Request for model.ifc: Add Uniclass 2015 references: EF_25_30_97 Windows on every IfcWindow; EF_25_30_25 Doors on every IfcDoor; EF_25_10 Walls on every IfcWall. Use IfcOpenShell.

First a look at what the model holds.

```python
import ifcopenshell

model = ifcopenshell.open("model.ifc")
print(model.schema)
print("classifications:", [c.Name for c in model.by_type("IfcClassification")])
for ifc_class in ("IfcDoor", "IfcRoof", "IfcStair", "IfcWall", "IfcWindow"):
    print(ifc_class, len(model.by_type(ifc_class)))
```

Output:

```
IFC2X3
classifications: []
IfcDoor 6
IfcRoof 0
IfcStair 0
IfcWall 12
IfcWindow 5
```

```python
import ifcopenshell
import ifcopenshell.api.classification

model = ifcopenshell.open("model.ifc")

# IFC2X3 requires Source and Edition and has no link from the project to the system.
system = model.create_entity("IfcClassification", Source="NBS", Edition="2015", Name="Uniclass 2015")

codes = {
    "IfcWindow": ("EF_25_30_97", "Windows"),
    "IfcDoor": ("EF_25_30_25", "Doors"),
    "IfcWall": ("EF_25_10", "Walls"),
}
for ifc_class, (code, name) in codes.items():
    products = model.by_type(ifc_class)
    ifcopenshell.api.classification.add_reference(
        model, products=products, classification=system, identification=code, name=name
    )
    print(code, len(products))

model.write("model_edited.ifc")
```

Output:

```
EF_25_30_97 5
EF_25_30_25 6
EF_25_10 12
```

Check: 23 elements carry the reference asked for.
